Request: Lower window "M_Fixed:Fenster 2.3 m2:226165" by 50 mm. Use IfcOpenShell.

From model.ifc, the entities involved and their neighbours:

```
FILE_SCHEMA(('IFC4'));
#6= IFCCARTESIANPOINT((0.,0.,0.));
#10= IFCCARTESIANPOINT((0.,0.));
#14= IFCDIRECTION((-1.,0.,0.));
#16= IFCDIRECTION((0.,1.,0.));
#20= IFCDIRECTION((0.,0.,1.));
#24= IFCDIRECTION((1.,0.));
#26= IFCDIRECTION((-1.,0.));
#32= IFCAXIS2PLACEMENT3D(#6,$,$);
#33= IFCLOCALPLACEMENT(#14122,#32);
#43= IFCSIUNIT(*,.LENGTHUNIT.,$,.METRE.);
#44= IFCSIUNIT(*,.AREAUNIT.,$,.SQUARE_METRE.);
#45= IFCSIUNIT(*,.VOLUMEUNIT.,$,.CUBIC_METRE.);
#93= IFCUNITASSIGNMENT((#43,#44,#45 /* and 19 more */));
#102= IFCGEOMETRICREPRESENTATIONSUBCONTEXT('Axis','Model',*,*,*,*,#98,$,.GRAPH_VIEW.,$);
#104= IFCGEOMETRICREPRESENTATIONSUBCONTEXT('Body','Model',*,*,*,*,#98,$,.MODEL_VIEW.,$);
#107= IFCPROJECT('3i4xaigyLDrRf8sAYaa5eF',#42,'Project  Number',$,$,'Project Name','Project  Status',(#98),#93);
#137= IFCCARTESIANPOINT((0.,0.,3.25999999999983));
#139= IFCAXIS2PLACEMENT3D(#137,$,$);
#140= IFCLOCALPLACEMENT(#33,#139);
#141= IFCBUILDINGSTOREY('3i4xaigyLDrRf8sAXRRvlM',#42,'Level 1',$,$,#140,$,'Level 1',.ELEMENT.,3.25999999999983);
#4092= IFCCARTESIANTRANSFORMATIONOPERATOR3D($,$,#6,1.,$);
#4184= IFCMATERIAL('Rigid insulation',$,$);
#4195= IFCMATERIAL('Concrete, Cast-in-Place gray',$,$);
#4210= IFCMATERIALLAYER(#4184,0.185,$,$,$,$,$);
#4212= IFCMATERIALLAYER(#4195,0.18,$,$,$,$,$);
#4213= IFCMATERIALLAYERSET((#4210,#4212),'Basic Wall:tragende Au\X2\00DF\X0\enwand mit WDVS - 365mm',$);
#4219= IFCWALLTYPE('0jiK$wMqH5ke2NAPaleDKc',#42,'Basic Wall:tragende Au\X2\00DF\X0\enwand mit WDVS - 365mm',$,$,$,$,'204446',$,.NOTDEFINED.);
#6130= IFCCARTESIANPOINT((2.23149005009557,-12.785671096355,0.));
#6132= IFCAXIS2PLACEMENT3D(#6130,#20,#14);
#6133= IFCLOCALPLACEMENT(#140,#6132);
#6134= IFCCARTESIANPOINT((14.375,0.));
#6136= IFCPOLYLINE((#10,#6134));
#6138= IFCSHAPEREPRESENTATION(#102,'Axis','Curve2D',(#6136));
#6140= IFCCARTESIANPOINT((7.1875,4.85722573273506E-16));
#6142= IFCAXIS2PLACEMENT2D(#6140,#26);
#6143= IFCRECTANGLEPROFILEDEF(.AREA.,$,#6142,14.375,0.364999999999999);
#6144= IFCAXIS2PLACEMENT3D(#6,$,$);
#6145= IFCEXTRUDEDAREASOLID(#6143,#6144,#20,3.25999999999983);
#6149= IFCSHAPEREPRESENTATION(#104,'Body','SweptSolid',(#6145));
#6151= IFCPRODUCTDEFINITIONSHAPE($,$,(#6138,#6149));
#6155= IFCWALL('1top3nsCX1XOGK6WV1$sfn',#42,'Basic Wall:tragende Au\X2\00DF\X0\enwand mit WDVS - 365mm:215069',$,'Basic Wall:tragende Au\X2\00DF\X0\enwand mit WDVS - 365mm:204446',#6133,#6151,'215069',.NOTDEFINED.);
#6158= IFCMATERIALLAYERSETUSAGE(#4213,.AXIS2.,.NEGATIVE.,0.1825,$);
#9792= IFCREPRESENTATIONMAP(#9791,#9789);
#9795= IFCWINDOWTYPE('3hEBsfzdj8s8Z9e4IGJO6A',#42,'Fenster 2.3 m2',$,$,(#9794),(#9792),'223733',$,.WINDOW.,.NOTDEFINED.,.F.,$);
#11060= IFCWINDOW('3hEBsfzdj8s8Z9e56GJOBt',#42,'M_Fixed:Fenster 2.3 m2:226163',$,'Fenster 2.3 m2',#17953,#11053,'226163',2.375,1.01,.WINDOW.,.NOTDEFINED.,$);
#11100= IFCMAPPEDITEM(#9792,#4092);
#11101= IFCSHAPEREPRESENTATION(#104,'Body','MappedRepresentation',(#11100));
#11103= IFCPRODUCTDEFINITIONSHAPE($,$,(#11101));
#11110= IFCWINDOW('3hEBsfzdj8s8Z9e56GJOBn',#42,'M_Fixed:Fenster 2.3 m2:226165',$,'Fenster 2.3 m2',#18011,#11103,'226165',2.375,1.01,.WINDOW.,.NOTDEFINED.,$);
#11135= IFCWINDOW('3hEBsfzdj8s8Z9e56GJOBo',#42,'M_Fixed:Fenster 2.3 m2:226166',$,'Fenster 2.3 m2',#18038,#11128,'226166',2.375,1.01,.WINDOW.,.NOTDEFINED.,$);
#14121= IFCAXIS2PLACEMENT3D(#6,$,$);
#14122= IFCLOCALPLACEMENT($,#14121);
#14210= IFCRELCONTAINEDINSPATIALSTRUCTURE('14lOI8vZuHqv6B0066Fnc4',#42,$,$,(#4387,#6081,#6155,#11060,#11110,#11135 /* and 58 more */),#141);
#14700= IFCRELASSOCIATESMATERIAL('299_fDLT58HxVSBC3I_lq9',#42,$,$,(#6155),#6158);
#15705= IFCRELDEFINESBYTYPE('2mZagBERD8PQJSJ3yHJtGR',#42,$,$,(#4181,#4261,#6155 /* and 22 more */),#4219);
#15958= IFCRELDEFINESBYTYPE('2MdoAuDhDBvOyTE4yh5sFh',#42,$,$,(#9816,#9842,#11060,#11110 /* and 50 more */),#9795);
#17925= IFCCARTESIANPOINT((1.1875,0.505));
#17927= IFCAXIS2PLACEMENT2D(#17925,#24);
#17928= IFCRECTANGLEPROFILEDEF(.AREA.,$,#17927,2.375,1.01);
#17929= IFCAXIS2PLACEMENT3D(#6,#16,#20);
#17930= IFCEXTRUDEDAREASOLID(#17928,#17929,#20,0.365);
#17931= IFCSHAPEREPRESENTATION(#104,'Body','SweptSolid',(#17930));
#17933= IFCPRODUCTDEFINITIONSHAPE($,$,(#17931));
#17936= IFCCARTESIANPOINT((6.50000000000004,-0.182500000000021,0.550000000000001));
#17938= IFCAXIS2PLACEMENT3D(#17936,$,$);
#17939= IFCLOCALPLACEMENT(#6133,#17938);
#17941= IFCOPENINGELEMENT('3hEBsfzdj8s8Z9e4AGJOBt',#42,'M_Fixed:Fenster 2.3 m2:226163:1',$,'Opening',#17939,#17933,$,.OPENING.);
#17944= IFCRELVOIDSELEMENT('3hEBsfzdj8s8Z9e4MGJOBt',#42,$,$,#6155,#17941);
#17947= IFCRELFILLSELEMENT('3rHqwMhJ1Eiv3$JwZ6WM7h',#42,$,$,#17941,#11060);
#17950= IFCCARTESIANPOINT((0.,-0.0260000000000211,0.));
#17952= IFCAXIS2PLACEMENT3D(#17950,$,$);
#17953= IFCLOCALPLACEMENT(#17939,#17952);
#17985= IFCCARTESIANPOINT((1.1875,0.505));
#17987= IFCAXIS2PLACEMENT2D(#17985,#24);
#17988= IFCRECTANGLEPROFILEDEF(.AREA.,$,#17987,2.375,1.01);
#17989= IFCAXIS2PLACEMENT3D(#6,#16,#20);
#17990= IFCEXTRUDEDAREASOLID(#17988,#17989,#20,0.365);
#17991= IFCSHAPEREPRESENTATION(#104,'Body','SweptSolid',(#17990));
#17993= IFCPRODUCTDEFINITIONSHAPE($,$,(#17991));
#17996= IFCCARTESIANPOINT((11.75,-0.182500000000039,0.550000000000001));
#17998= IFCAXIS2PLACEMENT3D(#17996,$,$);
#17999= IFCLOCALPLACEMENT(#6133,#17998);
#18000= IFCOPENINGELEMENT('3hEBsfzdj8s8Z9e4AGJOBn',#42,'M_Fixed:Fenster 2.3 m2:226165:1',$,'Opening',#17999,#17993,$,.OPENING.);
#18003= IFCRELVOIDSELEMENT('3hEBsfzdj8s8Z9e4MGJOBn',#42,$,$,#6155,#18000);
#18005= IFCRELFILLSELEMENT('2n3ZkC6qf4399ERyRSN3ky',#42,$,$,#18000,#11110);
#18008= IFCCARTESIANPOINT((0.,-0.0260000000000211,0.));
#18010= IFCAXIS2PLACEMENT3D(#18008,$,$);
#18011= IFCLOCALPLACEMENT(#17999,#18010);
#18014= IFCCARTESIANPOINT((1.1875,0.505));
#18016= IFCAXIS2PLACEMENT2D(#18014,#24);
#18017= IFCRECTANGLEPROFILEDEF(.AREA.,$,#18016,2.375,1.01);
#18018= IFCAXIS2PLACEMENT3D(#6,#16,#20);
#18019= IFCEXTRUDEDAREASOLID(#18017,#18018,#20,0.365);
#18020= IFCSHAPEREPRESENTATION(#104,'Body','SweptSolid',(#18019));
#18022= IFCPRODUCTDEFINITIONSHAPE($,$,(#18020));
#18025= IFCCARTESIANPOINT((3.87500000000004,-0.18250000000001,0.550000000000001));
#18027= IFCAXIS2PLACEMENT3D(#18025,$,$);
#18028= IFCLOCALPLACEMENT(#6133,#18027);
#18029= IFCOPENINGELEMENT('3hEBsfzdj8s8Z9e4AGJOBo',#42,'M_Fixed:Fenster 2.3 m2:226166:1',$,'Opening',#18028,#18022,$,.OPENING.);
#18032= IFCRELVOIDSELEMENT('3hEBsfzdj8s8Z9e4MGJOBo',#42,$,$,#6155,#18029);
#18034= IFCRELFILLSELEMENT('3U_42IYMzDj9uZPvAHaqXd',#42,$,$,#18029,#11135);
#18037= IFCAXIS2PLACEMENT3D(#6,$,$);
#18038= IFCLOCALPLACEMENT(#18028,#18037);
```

```python
import numpy as np
import ifcopenshell
import ifcopenshell.api.geometry
import ifcopenshell.util.placement
import ifcopenshell.util.unit

model = ifcopenshell.open("model.ifc")
unit_scale = ifcopenshell.util.unit.calculate_unit_scale(model)

window = model.by_guid("3hEBsfzdj8s8Z9e56GJOBn")
opening = window.FillsVoids[0].RelatingOpeningElement
dz = -0.05 / unit_scale

shift = np.array([0.0, 0.0, dz])
# The window is placed relative to its opening, so it follows when the opening moves.
matrix = ifcopenshell.util.placement.get_local_placement(opening.ObjectPlacement)
matrix[:3, 3] += shift
ifcopenshell.api.geometry.edit_object_placement(
    model, product=opening, matrix=matrix, is_si=False, should_transform_children=True
)

print(f"moved by {dz * unit_scale:+.3f} m")

model.write("model-out.ifc")
```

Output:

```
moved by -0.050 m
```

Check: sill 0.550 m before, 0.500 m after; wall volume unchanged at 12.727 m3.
